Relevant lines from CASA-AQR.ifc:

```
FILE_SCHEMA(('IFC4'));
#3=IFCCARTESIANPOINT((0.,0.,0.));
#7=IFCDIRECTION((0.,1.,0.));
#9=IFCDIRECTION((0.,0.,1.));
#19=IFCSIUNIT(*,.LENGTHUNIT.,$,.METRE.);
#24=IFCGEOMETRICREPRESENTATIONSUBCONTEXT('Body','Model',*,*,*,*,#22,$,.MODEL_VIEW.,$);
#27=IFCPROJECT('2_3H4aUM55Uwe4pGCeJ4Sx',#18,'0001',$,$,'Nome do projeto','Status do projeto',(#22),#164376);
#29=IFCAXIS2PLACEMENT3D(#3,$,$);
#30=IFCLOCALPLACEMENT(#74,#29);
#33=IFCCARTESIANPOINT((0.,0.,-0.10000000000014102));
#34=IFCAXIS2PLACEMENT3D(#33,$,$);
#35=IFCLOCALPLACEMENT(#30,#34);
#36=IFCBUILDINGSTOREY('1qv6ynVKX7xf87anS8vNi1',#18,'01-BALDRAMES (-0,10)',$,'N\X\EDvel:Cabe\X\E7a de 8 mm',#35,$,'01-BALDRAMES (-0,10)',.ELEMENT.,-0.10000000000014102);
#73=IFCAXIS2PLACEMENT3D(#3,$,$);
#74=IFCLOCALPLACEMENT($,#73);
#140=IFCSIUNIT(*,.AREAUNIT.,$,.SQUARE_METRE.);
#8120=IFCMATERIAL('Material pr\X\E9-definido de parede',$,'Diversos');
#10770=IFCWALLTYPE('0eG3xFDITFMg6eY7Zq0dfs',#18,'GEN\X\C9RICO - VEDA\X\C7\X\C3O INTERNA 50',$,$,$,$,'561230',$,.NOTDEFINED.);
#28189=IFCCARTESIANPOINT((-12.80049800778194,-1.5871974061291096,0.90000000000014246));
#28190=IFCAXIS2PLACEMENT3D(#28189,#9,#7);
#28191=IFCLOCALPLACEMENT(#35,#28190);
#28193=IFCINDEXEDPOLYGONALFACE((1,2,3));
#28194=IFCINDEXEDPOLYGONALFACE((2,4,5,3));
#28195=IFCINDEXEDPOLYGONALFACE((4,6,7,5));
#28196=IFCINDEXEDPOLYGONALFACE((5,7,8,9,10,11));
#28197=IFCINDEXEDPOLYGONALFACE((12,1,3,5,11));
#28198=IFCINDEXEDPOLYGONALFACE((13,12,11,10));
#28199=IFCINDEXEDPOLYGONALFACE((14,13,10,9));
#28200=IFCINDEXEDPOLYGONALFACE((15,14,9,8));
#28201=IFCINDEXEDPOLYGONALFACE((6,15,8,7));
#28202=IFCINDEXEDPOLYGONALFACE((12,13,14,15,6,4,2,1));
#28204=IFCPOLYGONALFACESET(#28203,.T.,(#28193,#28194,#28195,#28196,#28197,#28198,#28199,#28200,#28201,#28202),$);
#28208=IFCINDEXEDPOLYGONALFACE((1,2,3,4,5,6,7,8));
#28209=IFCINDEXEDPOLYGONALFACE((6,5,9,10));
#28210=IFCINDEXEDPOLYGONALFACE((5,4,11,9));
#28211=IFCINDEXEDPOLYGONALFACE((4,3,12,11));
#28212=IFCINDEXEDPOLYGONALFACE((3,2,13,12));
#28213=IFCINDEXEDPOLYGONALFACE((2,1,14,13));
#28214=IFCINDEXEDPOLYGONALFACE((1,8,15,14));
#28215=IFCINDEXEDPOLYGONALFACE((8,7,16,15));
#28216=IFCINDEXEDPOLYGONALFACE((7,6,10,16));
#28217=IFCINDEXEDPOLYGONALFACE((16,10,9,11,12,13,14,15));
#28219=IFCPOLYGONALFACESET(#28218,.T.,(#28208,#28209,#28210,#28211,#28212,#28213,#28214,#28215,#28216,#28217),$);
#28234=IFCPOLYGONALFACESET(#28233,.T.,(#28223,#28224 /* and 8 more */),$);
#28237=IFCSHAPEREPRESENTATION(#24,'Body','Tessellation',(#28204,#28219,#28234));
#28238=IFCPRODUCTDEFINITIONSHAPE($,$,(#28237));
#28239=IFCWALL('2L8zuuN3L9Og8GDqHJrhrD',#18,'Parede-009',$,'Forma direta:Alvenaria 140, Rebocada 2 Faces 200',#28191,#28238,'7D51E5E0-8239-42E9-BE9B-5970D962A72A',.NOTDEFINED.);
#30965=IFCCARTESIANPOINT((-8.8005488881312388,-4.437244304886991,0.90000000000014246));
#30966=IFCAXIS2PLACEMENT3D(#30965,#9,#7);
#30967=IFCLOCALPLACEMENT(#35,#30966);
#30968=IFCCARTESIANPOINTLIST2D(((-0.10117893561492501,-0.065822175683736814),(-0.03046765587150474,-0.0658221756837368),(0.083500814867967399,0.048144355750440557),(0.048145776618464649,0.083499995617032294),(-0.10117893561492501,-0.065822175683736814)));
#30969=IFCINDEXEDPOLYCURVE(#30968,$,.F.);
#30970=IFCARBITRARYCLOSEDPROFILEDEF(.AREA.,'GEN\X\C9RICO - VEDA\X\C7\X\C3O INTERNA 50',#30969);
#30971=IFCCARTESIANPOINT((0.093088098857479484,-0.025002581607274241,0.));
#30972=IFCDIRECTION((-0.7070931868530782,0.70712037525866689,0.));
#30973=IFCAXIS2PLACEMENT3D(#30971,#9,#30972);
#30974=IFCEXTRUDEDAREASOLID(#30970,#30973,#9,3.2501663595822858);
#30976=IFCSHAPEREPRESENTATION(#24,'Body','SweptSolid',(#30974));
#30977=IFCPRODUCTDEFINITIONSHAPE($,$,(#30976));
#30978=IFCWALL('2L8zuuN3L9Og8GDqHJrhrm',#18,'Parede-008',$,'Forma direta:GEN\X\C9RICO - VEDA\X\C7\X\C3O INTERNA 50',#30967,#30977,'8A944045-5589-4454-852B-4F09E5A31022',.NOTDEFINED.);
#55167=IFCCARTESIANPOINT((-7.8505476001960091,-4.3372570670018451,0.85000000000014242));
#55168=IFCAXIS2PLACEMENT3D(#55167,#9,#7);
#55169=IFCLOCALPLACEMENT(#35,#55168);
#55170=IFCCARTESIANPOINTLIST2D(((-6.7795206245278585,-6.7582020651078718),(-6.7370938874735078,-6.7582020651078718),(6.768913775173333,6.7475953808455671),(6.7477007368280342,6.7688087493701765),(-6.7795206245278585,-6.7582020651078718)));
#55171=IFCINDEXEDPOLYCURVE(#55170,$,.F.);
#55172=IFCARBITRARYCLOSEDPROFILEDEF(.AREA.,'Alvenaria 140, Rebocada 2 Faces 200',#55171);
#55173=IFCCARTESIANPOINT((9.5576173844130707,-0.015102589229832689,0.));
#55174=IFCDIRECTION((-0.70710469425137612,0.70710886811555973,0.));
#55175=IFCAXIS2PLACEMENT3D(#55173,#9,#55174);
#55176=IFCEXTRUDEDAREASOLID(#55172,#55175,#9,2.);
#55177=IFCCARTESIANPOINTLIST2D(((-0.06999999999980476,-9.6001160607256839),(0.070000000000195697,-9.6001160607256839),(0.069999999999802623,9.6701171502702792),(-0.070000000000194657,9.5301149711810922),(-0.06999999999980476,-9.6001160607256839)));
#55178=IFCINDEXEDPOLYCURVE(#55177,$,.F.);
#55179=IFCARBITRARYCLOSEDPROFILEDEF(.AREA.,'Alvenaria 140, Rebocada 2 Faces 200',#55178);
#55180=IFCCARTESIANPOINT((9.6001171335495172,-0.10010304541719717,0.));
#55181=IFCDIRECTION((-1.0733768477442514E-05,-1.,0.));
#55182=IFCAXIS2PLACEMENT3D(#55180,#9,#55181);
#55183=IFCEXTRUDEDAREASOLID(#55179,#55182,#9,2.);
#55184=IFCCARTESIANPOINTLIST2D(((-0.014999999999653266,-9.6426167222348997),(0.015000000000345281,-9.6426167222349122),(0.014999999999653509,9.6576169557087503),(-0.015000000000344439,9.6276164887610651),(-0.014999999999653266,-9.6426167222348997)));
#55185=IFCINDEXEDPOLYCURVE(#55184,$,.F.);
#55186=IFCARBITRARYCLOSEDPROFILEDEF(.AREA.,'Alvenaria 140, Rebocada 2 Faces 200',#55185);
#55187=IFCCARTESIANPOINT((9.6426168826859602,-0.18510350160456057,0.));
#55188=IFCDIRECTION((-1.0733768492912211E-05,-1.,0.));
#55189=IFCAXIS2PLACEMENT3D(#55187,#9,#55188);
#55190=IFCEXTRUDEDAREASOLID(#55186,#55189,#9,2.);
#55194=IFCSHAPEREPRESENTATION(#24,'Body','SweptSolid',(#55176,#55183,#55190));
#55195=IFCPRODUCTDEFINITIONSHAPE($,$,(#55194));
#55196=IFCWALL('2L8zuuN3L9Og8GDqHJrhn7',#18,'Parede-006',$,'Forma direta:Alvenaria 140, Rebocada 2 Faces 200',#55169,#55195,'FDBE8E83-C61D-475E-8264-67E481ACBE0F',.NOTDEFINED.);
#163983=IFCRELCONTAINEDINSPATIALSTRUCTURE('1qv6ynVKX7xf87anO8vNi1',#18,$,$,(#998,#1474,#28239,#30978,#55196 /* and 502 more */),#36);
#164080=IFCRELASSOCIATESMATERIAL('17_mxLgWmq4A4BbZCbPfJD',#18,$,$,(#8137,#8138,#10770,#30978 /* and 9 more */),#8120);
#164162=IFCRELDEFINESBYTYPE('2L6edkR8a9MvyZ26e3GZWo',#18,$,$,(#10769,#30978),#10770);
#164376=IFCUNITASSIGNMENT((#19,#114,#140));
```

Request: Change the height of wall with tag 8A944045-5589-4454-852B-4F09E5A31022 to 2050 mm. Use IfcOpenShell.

```python
import ifcopenshell
import ifcopenshell.geom
import ifcopenshell.util.representation
import ifcopenshell.util.shape
import ifcopenshell.util.unit

model = ifcopenshell.open("CASA-AQR.ifc")
unit_scale = ifcopenshell.util.unit.calculate_unit_scale(model)
settings = ifcopenshell.geom.settings()


def volume(element):
    """Net volume in cubic metres, openings subtracted."""
    shape = ifcopenshell.geom.create_shape(settings, element)
    return ifcopenshell.util.shape.get_volume(shape.geometry)


wall = model.by_id(30978)
before = volume(wall)

body = ifcopenshell.util.representation.get_representation(wall, "Model", "Body")
solid = body.Items[0]
old_height = solid.Depth
solid.Depth = 2.05 / unit_scale
after = volume(wall)

print(f"height {old_height:g} -> {solid.Depth:g}, volume {before:.3f} -> {after:.3f} m3")

model.write("CASA-AQR_v2.ifc")
```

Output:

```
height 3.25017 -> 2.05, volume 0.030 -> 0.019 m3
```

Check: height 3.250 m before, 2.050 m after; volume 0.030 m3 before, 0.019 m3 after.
